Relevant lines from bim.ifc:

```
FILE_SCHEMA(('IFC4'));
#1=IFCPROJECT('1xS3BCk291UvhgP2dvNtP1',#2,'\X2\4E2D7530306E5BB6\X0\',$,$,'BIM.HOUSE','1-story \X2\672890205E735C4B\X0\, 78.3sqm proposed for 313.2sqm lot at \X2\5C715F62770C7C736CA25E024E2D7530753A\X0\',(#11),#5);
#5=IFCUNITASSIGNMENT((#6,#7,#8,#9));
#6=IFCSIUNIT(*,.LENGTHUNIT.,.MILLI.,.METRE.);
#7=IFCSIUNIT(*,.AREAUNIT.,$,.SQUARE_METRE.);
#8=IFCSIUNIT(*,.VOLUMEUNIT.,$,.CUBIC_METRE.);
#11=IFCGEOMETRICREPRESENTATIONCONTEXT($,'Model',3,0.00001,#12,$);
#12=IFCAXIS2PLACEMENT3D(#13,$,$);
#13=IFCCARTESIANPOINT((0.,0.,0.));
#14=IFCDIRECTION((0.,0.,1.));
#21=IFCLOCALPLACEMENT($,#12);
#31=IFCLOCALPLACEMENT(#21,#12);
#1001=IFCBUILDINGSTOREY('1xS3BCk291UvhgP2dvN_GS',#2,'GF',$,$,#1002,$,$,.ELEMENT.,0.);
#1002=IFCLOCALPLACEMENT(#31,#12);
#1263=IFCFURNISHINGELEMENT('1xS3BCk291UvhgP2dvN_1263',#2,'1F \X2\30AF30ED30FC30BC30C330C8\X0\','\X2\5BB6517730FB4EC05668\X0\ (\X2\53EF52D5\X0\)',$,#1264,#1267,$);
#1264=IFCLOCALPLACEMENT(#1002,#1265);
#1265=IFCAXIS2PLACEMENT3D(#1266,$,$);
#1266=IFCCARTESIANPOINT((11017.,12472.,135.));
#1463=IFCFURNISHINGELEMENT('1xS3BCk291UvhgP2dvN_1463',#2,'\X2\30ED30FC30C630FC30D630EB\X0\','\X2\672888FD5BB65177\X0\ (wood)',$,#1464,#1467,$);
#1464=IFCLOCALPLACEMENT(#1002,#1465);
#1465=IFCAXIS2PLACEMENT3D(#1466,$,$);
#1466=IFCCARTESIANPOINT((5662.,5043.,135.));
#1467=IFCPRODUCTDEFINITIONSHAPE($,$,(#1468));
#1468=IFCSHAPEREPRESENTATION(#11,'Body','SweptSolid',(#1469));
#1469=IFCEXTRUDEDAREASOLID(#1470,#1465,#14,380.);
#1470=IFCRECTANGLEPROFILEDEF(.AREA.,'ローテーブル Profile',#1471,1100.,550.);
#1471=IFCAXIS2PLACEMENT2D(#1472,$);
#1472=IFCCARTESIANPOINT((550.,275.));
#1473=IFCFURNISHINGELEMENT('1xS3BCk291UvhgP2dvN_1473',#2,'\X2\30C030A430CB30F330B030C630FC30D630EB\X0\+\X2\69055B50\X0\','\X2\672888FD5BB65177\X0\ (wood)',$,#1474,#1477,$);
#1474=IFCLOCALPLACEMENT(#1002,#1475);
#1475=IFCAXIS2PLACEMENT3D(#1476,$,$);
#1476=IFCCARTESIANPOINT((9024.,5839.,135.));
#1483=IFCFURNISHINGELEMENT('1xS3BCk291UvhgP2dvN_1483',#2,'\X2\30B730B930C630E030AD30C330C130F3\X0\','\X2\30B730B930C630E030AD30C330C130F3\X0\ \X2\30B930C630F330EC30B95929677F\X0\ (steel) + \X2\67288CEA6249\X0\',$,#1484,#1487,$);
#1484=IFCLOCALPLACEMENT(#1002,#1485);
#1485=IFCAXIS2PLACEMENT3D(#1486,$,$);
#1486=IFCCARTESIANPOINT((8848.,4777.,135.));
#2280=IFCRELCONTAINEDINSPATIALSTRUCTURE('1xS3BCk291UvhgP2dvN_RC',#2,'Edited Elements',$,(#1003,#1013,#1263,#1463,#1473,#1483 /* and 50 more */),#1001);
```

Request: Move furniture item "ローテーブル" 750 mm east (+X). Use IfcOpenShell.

```python
import ifcopenshell
import ifcopenshell.api.geometry
import ifcopenshell.util.placement
import ifcopenshell.util.unit

model = ifcopenshell.open("bim.ifc")
unit_scale = ifcopenshell.util.unit.calculate_unit_scale(model)

item = model.by_guid("1xS3BCk291UvhgP2dvN_1463")
matrix = ifcopenshell.util.placement.get_local_placement(item.ObjectPlacement)
matrix[0, 3] += 0.75 / unit_scale
ifcopenshell.api.geometry.edit_object_placement(model, product=item, matrix=matrix, is_si=False)

print(ifcopenshell.util.placement.get_local_placement(item.ObjectPlacement).round(3) + 0.0)

model.write("bim_rev.ifc")
```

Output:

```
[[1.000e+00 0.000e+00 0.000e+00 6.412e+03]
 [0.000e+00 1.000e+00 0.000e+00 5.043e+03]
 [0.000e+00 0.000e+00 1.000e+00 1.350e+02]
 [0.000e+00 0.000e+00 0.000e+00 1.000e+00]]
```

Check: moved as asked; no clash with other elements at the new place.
